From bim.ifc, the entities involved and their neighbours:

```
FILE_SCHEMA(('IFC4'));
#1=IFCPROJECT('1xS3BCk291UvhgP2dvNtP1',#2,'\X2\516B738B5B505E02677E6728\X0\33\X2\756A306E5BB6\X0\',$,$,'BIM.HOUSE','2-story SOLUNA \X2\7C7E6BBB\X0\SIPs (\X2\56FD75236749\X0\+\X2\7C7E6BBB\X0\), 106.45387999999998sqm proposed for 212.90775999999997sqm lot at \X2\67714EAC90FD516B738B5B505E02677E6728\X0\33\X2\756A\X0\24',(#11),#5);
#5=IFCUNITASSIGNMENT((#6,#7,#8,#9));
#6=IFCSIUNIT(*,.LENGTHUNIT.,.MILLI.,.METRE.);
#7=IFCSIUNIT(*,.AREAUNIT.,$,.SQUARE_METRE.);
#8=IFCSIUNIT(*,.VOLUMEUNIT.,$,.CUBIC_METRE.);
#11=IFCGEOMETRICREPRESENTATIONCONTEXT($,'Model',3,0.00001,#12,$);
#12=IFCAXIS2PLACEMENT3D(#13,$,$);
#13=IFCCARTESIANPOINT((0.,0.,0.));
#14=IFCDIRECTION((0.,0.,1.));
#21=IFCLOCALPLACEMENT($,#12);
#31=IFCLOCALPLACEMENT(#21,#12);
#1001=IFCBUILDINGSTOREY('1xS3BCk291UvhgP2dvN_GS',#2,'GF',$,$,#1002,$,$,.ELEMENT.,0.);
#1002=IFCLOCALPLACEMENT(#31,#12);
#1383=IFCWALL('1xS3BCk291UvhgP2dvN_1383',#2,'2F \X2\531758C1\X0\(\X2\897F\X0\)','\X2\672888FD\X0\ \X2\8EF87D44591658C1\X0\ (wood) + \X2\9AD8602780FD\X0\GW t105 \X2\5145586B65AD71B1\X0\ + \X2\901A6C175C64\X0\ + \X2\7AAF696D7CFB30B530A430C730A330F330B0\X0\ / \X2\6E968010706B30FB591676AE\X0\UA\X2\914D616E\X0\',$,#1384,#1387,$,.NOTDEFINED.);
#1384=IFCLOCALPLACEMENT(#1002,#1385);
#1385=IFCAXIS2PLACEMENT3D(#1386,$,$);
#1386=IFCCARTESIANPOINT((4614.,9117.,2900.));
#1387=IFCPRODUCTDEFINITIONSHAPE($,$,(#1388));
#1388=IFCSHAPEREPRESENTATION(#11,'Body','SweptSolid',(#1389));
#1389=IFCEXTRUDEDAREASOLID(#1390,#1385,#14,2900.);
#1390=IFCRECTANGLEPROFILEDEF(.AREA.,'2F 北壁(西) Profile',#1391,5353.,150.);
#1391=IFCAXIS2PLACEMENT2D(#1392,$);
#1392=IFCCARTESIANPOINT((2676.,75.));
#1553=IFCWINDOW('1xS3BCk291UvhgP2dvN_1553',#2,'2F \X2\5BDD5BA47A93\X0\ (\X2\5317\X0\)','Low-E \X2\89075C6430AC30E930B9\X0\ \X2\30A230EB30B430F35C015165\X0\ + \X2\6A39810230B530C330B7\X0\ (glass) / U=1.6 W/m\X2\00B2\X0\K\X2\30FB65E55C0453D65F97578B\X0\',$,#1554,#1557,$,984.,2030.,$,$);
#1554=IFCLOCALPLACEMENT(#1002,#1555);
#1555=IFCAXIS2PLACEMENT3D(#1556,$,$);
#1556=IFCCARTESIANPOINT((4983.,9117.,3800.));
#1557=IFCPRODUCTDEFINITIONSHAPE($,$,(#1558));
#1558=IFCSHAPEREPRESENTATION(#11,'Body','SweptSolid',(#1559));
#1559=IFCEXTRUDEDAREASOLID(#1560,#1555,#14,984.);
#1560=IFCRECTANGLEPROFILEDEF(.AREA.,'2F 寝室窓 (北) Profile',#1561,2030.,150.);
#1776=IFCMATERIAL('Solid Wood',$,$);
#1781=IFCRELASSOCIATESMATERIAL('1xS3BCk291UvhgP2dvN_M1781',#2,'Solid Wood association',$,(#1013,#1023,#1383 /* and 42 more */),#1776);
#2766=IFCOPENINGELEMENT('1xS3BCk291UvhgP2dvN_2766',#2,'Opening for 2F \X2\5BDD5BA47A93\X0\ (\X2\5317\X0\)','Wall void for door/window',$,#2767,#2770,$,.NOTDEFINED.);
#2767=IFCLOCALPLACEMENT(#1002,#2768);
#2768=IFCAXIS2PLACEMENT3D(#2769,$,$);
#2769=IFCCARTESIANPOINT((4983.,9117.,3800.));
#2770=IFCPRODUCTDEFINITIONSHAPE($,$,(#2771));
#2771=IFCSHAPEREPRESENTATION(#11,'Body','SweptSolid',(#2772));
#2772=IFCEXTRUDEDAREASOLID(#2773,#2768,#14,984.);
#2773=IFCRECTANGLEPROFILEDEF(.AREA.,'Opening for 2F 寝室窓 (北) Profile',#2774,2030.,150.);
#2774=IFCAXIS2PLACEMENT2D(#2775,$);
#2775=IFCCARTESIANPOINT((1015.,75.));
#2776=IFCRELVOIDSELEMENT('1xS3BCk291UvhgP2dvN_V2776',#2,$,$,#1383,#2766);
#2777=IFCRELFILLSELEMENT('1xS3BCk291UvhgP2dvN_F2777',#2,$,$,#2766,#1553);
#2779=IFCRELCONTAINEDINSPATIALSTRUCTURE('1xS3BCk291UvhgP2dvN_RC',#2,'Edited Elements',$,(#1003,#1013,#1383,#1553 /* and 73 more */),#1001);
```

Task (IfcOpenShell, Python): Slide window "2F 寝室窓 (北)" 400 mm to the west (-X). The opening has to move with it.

```python
import ifcopenshell
import ifcopenshell.api.geometry
import ifcopenshell.util.placement
import ifcopenshell.util.unit

model = ifcopenshell.open("bim.ifc")
unit_scale = ifcopenshell.util.unit.calculate_unit_scale(model)

window = model.by_guid("1xS3BCk291UvhgP2dvN_1553")
opening = window.FillsVoids[0].RelatingOpeningElement
wall = opening.VoidsElements[0].RelatingBuildingElement

wall_matrix = ifcopenshell.util.placement.get_local_placement(wall.ObjectPlacement)
shift = wall_matrix[:3, 0] * -0.4 / unit_scale
before = ifcopenshell.util.placement.get_local_placement(window.ObjectPlacement)[:3, 3].copy()

# The window is not placed relative to its opening, so move both.
for product in (opening, window):
    matrix = ifcopenshell.util.placement.get_local_placement(product.ObjectPlacement)
    matrix[:3, 3] += shift
    ifcopenshell.api.geometry.edit_object_placement(model, product=product, matrix=matrix, is_si=False)

after = ifcopenshell.util.placement.get_local_placement(window.ObjectPlacement)[:3, 3]
print("window moved by", (after - before).round(3) + 0.0)

model.write("bim_updated.ifc")
```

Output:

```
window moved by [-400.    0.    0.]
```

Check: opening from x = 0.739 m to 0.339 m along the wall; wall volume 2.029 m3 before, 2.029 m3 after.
